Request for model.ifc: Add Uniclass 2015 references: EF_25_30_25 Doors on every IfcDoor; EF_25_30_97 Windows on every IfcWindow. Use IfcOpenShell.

First a look at what the model holds.

```python
import ifcopenshell

model = ifcopenshell.open("model.ifc")
print(model.schema)
print("classifications:", [c.Name for c in model.by_type("IfcClassification")])
for ifc_class in ("IfcDoor", "IfcRoof", "IfcStair", "IfcWall", "IfcWindow"):
    print(ifc_class, len(model.by_type(ifc_class)))
```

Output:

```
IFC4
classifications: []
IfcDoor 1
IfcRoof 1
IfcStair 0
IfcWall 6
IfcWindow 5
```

```python
import ifcopenshell
import ifcopenshell.api.classification

model = ifcopenshell.open("model.ifc")

system = ifcopenshell.api.classification.add_classification(model, classification="Uniclass 2015")

codes = {
    "IfcDoor": ("EF_25_30_25", "Doors"),
    "IfcWindow": ("EF_25_30_97", "Windows"),
}
for ifc_class, (code, name) in codes.items():
    products = model.by_type(ifc_class)
    ifcopenshell.api.classification.add_reference(
        model, products=products, classification=system, identification=code, name=name
    )
    print(code, len(products))

model.write("model-out.ifc")
```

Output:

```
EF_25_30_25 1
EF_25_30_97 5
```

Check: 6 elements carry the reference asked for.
